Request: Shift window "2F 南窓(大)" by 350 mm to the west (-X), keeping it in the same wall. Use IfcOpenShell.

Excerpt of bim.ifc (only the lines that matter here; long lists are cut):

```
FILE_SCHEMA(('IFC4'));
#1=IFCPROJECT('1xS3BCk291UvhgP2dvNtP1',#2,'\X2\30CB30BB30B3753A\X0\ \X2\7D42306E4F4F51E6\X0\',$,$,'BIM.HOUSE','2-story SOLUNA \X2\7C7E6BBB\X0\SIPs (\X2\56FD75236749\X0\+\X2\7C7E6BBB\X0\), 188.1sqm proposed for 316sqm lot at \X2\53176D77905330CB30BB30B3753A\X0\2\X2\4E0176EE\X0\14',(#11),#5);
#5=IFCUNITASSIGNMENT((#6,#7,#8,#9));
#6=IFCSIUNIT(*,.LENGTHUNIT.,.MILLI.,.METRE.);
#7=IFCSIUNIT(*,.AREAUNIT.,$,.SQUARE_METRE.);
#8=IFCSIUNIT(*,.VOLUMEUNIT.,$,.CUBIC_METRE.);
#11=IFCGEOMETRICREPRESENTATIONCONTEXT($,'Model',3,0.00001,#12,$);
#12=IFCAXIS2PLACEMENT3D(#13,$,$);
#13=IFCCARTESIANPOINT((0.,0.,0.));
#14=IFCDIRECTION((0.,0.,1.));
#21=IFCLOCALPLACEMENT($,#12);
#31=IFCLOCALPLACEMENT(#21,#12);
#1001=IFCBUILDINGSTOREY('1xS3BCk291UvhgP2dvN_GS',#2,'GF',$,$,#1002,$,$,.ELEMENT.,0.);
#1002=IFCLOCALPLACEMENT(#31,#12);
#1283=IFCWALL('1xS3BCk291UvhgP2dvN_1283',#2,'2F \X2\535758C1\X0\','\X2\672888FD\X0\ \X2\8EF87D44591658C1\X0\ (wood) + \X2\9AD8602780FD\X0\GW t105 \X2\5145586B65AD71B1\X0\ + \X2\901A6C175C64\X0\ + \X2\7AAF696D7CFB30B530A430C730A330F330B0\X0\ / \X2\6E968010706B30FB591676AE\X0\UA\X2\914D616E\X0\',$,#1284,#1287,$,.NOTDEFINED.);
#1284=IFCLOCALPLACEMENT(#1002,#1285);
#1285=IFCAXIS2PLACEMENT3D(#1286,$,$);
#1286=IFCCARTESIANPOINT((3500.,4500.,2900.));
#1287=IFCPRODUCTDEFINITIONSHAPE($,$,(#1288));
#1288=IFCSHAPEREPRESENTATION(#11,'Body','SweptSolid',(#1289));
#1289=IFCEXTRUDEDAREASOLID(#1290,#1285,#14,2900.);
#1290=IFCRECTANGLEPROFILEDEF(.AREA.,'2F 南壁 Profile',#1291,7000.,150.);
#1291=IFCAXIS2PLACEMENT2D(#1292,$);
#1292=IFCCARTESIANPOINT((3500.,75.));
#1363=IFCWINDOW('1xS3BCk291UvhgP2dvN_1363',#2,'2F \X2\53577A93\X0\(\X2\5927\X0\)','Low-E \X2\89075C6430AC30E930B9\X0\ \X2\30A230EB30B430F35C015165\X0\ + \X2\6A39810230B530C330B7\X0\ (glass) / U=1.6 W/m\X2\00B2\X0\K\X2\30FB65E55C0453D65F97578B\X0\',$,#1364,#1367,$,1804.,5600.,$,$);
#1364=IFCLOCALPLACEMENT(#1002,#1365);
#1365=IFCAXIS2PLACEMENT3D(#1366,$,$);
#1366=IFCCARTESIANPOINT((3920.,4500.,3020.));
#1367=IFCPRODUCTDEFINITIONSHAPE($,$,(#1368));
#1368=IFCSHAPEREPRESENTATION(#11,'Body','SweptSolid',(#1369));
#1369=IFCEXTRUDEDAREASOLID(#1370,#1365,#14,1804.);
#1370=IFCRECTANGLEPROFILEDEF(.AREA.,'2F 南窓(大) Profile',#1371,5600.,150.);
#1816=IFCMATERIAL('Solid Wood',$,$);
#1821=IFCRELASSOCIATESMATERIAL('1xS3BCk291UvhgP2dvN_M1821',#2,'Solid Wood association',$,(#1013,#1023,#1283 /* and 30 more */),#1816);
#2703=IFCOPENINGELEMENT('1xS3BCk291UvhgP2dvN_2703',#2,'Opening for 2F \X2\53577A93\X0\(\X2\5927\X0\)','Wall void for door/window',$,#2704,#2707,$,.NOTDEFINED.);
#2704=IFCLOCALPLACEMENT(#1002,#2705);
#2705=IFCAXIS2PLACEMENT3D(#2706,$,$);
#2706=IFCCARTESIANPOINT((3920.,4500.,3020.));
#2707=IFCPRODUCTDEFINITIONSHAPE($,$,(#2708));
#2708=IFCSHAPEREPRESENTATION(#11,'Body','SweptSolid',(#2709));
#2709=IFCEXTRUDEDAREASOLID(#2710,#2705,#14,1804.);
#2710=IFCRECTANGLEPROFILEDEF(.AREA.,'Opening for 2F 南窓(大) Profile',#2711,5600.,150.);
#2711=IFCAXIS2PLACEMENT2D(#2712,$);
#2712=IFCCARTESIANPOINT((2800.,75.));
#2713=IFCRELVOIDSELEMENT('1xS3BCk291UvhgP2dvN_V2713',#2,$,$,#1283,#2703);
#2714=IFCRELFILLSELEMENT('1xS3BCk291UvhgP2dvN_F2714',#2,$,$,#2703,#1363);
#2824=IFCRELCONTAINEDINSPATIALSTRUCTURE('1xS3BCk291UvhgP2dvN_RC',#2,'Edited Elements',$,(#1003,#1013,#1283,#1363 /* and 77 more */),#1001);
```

```python
import ifcopenshell
import ifcopenshell.api.geometry
import ifcopenshell.util.placement
import ifcopenshell.util.unit

model = ifcopenshell.open("bim.ifc")
unit_scale = ifcopenshell.util.unit.calculate_unit_scale(model)

window = model.by_guid("1xS3BCk291UvhgP2dvN_1363")
opening = window.FillsVoids[0].RelatingOpeningElement
wall = opening.VoidsElements[0].RelatingBuildingElement

wall_matrix = ifcopenshell.util.placement.get_local_placement(wall.ObjectPlacement)
shift = wall_matrix[:3, 0] * -0.35 / unit_scale
before = ifcopenshell.util.placement.get_local_placement(window.ObjectPlacement)[:3, 3].copy()

# The window is not placed relative to its opening, so move both.
for product in (opening, window):
    matrix = ifcopenshell.util.placement.get_local_placement(product.ObjectPlacement)
    matrix[:3, 3] += shift
    ifcopenshell.api.geometry.edit_object_placement(model, product=product, matrix=matrix, is_si=False)

after = ifcopenshell.util.placement.get_local_placement(window.ObjectPlacement)[:3, 3]
print("window moved by", (after - before).round(3) + 0.0)

model.write("bim_v2.ifc")
```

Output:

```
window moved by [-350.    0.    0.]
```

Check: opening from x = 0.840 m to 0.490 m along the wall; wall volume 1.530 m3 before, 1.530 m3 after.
